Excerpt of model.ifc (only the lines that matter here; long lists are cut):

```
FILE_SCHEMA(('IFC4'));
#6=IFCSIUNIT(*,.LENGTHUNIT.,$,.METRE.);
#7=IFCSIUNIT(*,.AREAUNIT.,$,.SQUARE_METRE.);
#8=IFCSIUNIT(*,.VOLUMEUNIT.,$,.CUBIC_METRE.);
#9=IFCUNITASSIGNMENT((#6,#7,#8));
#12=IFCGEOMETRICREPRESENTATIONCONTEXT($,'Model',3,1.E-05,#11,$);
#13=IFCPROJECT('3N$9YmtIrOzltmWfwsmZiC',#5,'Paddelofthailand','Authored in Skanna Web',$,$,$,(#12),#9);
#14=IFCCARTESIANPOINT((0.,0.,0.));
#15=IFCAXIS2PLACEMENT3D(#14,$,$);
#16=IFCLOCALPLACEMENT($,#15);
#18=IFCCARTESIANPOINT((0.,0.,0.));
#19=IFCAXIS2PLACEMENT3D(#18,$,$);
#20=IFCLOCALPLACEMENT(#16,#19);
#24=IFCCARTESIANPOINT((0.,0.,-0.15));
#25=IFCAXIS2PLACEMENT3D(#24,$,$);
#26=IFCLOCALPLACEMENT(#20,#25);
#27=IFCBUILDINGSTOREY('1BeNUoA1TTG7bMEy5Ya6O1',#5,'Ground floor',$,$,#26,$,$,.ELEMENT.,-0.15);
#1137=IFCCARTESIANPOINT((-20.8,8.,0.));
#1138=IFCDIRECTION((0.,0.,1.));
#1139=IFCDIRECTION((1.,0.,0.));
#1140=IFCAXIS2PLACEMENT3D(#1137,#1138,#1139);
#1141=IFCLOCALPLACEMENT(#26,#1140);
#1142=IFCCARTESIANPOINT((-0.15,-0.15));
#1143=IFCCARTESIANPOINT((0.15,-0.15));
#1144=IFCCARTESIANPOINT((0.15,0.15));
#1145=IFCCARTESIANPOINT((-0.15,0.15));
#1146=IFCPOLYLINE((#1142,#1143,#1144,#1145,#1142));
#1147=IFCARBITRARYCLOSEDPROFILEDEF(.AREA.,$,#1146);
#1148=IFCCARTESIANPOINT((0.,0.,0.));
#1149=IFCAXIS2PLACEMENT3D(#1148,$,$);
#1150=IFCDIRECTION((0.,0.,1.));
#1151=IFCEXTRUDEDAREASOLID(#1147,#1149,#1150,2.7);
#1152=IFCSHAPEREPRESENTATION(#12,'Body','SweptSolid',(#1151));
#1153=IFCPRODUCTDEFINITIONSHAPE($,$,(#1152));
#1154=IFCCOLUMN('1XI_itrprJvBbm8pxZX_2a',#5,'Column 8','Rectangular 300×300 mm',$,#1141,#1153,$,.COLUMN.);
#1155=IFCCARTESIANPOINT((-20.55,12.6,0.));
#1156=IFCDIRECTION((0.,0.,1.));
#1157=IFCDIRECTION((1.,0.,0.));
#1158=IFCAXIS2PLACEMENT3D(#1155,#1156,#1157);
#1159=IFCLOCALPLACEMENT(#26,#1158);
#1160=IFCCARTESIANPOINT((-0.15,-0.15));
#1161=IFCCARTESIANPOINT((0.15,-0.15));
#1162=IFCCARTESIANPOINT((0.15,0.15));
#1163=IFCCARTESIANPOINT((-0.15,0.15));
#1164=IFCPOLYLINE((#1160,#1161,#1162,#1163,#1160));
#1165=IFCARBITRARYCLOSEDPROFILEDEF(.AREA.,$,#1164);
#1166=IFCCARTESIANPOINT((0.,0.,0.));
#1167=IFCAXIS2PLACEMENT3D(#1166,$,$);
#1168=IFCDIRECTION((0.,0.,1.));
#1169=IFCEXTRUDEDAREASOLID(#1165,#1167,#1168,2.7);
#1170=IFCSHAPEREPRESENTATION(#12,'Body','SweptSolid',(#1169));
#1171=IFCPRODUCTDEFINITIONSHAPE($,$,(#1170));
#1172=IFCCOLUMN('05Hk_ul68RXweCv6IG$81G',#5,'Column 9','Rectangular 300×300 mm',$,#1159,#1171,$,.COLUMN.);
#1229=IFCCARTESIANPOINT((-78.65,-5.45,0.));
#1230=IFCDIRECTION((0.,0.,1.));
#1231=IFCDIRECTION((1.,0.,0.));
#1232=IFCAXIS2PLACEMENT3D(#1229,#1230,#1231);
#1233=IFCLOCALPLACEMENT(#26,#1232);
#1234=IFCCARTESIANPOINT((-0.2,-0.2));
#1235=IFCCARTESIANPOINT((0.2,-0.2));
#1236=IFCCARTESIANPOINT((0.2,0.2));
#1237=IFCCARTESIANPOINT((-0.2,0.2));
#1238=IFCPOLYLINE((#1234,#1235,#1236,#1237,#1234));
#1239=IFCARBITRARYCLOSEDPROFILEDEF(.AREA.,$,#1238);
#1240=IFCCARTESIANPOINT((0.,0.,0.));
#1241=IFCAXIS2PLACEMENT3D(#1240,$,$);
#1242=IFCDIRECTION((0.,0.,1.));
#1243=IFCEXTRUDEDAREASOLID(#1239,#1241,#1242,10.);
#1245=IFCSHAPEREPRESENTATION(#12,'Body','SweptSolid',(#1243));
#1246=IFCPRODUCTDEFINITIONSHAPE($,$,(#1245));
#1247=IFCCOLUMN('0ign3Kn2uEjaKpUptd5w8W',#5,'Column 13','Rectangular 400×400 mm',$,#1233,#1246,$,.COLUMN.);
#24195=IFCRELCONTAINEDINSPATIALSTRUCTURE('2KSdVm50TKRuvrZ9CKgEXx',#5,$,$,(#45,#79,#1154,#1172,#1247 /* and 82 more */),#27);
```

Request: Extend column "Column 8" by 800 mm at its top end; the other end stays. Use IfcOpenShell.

```python
import ifcopenshell

model = ifcopenshell.open("model.ifc")

member = model.by_guid("1XI_itrprJvBbm8pxZX_2a")
change = 0.8

# The extrusion runs towards the end named, so only its depth changes.
body = next(r for r in member.Representation.Representations if r.RepresentationIdentifier == "Body")
solid = body.Items[0]
old_length = solid.Depth
solid.Depth += change

print(f"length {old_length:g} -> {solid.Depth:g}")

model.write("model-out.ifc")
```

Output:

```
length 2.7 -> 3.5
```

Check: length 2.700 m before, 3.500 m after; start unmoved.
